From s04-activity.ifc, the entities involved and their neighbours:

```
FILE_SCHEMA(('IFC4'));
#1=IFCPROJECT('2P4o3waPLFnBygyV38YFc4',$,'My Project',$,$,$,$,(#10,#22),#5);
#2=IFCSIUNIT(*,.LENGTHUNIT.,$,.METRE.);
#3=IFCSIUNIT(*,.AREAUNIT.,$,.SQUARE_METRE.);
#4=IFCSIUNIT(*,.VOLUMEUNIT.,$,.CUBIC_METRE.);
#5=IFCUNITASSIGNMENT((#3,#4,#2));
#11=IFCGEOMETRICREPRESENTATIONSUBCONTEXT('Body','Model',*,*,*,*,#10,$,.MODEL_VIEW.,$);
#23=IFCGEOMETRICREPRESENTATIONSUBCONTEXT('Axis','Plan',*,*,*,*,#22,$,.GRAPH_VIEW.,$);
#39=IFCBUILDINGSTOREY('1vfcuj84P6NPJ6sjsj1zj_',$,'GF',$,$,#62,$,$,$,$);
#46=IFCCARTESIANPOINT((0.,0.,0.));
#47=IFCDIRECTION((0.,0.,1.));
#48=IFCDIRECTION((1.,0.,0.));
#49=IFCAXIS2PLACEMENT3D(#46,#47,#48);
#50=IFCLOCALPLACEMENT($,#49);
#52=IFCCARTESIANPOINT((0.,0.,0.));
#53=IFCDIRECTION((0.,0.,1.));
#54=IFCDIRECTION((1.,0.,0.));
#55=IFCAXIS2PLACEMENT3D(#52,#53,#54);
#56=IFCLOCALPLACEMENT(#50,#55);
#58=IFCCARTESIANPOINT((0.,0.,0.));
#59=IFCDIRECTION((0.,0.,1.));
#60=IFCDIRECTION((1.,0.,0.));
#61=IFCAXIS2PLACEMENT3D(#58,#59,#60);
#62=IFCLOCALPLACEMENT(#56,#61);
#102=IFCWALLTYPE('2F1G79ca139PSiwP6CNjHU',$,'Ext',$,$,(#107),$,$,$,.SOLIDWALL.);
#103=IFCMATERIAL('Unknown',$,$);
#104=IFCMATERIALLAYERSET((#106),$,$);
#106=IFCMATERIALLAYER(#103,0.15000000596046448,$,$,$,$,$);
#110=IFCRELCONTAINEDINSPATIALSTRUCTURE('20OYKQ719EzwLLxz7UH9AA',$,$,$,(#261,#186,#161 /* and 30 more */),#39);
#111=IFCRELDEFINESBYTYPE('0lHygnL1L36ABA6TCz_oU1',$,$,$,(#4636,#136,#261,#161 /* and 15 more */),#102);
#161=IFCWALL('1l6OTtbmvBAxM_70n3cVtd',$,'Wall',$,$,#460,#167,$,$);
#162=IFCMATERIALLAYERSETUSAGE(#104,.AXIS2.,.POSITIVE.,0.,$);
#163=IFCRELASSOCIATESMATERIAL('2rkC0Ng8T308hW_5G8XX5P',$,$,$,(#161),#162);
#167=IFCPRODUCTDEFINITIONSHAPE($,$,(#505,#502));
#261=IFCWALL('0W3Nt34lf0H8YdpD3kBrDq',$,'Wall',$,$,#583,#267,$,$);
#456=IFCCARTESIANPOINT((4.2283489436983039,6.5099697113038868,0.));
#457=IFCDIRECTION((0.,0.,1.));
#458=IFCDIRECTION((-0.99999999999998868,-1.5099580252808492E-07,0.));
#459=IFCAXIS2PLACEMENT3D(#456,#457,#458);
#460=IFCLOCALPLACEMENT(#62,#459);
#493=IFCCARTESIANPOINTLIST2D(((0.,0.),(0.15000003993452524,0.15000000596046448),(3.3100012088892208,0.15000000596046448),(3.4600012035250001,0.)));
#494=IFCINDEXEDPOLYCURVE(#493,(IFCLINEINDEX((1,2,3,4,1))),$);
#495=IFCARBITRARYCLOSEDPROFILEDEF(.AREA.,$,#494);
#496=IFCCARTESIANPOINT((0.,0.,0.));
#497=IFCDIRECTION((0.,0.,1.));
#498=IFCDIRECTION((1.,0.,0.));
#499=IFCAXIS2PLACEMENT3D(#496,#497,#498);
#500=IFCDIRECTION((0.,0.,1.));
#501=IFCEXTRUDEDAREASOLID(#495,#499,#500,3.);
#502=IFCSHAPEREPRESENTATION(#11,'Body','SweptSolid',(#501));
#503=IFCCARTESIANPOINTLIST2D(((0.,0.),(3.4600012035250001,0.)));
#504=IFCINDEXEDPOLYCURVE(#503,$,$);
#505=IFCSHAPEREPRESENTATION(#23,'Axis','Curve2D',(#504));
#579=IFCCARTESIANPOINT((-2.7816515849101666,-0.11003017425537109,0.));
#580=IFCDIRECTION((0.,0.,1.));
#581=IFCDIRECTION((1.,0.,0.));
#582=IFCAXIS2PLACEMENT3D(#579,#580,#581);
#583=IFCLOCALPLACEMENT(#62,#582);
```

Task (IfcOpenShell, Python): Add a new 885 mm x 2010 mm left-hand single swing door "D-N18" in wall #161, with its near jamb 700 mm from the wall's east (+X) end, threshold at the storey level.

```python
import numpy as np
import ifcopenshell
import ifcopenshell.api.feature
import ifcopenshell.api.geometry
import ifcopenshell.api.root
import ifcopenshell.api.spatial
import ifcopenshell.geom
import ifcopenshell.util.element
import ifcopenshell.util.placement
import ifcopenshell.util.representation
import ifcopenshell.util.shape
import ifcopenshell.util.unit

model = ifcopenshell.open("s04-activity.ifc")
unit_scale = ifcopenshell.util.unit.calculate_unit_scale(model)
settings = ifcopenshell.geom.settings()


def volume(element):
    """Net volume in cubic metres, openings subtracted."""
    shape = ifcopenshell.geom.create_shape(settings, element)
    return ifcopenshell.util.shape.get_volume(shape.geometry)


wall = model.by_id(161)
storey = ifcopenshell.util.element.get_container(wall, ifc_class="IfcBuildingStorey")
context = ifcopenshell.util.representation.get_context(model, "Model", "Body", "MODEL_VIEW")
before = volume(wall)

width, height, from_end, sill = 0.885, 2.01, 0.7, 0.0  # metres

# The wall runs along its own X axis, and the end named is its -X end.
wall_shape = ifcopenshell.geom.create_shape(settings, wall)
x, y, z = ifcopenshell.util.shape.get_vertices(wall_shape.geometry).T
start = x.min() + from_end
face, thickness = float(y.min()), float(y.max() - y.min())
wall_matrix = ifcopenshell.util.placement.get_local_placement(wall.ObjectPlacement)
level = ifcopenshell.util.placement.get_local_placement(storey.ObjectPlacement)[2, 3]


def in_wall(x, y):
    """Placement at x, y metres in the wall's axes, at sill height."""
    matrix = wall_matrix.copy()
    matrix[:, 3] = wall_matrix @ np.array([x / unit_scale, y / unit_scale, 0.0, 1.0])
    matrix[2, 3] = level + sill / unit_scale
    return matrix


# Opening: a box that overshoots both wall faces by 50 mm.
opening = ifcopenshell.api.root.create_entity(model, ifc_class="IfcOpeningElement", predefined_type="OPENING")
box = ifcopenshell.api.geometry.add_wall_representation(
    model, context=context, length=width, height=height, thickness=thickness + 0.1
)
ifcopenshell.api.geometry.assign_representation(model, product=opening, representation=box)
ifcopenshell.api.geometry.edit_object_placement(model, product=opening, matrix=in_wall(start, face - 0.05), is_si=False)
ifcopenshell.api.feature.add_feature(model, feature=opening, element=wall)

door = ifcopenshell.api.root.create_entity(model, ifc_class="IfcDoor", name="D-N18", predefined_type="DOOR")
door.OverallWidth, door.OverallHeight = width / unit_scale, height / unit_scale
door.OperationType = "SINGLE_SWING_LEFT"
body = ifcopenshell.api.geometry.add_door_representation(
    model,
    context=context,
    overall_width=door.OverallWidth,
    overall_height=door.OverallHeight,
    operation_type="SINGLE_SWING_LEFT",
    lining_properties={"LiningDepth": thickness / unit_scale, "ThresholdDepth": thickness / unit_scale},
)
ifcopenshell.api.geometry.assign_representation(model, product=door, representation=body)
ifcopenshell.api.spatial.assign_container(model, products=[door], relating_structure=storey)
ifcopenshell.api.feature.add_filling(model, opening=opening, element=door)

# The lining spans the wall, so the door starts at the wall face.
ifcopenshell.api.geometry.edit_object_placement(model, product=door, matrix=in_wall(start, face), is_si=False)

after = volume(wall)

print(f"wall volume {before:.3f} -> {after:.3f} m3")

model.write("s04-activity_v2.ifc")
```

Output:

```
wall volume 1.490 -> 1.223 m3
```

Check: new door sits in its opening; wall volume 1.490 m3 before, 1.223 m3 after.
